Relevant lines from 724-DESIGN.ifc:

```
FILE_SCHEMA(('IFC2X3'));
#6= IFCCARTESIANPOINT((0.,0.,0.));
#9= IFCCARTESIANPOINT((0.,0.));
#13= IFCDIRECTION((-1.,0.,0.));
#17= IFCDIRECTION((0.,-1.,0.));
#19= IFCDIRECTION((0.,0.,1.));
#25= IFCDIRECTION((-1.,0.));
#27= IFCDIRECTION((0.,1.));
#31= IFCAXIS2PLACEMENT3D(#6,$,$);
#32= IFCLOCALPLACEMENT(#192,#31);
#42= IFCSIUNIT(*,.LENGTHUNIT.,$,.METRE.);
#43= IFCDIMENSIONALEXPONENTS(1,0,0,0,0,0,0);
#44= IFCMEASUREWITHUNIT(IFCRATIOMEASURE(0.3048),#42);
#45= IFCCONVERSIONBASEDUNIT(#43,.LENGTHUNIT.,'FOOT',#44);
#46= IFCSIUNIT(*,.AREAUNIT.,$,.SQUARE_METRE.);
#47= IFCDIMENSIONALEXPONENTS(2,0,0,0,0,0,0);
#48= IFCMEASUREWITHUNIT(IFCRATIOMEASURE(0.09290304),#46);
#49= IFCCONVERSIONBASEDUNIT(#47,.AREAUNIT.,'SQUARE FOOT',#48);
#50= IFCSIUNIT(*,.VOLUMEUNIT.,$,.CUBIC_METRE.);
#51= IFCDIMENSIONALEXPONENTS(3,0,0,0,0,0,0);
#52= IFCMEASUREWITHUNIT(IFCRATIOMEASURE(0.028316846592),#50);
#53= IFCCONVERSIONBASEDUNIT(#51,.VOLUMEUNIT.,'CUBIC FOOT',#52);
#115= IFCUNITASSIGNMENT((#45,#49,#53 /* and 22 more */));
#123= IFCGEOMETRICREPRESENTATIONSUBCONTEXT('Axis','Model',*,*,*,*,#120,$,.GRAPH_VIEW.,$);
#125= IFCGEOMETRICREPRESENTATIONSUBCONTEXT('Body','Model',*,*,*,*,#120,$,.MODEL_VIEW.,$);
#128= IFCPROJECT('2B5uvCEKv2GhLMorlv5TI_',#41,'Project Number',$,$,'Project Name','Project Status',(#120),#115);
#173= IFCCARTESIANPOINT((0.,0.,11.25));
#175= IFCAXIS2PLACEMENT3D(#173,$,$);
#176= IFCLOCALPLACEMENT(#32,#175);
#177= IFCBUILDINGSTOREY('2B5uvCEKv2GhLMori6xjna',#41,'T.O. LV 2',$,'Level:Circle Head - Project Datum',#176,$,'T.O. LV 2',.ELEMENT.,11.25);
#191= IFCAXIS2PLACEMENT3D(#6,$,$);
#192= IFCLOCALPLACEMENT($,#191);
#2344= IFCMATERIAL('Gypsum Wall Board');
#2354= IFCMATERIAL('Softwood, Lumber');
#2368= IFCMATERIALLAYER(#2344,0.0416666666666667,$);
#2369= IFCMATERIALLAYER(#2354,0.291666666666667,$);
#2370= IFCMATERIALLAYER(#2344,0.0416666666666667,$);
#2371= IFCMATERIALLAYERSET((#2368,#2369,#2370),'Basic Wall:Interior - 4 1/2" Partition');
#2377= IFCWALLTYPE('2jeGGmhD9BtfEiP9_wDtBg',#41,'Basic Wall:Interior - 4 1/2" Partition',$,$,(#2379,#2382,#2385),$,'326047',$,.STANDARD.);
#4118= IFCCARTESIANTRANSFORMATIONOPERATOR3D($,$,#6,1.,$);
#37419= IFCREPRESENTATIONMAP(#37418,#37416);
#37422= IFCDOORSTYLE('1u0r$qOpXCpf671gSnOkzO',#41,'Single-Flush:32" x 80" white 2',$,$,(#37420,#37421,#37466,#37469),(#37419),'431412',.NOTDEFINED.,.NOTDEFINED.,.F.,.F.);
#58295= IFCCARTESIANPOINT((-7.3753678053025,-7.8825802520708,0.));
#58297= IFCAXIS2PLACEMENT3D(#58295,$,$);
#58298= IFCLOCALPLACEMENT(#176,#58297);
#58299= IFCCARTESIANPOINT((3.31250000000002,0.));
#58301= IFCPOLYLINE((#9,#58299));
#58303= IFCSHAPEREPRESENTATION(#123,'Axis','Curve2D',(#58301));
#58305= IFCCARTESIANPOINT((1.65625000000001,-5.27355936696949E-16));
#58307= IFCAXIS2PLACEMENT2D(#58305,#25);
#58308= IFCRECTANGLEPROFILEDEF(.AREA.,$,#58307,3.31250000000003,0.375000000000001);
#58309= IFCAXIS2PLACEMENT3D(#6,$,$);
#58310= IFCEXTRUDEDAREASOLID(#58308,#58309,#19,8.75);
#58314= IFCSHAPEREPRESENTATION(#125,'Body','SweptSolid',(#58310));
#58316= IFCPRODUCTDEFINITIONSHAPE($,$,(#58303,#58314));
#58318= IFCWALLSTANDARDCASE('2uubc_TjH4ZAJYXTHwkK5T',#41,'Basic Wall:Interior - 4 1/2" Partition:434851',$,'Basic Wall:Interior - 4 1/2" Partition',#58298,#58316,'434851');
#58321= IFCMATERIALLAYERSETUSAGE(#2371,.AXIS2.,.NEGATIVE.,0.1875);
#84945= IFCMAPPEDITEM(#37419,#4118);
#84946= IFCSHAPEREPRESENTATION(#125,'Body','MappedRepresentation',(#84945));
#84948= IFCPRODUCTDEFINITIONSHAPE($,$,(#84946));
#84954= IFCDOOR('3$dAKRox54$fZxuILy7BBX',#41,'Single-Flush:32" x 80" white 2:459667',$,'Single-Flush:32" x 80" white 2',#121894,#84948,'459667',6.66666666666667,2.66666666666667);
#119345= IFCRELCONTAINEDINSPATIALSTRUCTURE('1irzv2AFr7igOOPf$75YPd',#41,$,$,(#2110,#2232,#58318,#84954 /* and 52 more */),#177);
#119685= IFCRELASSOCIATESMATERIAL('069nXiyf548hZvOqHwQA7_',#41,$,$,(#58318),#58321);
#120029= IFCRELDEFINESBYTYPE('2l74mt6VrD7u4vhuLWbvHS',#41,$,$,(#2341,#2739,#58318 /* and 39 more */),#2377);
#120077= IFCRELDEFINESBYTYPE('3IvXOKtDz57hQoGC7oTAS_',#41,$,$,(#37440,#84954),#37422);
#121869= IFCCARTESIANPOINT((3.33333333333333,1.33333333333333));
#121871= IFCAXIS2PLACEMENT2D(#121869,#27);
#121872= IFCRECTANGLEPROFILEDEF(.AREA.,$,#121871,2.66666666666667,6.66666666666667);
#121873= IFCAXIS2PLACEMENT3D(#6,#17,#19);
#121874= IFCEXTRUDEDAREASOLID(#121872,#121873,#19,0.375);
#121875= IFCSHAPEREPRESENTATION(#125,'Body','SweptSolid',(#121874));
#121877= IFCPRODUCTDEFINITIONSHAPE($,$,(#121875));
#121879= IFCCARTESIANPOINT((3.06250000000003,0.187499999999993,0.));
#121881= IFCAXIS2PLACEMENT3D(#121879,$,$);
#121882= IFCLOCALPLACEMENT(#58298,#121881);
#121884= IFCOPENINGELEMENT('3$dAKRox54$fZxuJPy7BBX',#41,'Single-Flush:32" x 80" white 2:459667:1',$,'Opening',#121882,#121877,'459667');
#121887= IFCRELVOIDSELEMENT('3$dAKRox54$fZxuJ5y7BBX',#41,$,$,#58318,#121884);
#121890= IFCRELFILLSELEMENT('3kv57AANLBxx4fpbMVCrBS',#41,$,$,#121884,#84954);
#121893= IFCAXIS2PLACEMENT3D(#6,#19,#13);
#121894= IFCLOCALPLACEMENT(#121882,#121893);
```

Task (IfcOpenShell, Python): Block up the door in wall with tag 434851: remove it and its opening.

```python
import ifcopenshell
import ifcopenshell.api.feature
import ifcopenshell.api.root
import ifcopenshell.geom
import ifcopenshell.util.shape

model = ifcopenshell.open("724-DESIGN.ifc")
settings = ifcopenshell.geom.settings()


def volume(element):
    """Net volume in cubic metres, openings subtracted."""
    shape = ifcopenshell.geom.create_shape(settings, element)
    return ifcopenshell.util.shape.get_volume(shape.geometry)


door = model.by_guid("3$dAKRox54$fZxuILy7BBX")
opening = door.FillsVoids[0].RelatingOpeningElement
wall = opening.VoidsElements[0].RelatingBuildingElement
before = volume(wall)

ifcopenshell.api.root.remove_product(model, product=door)
ifcopenshell.api.feature.remove_feature(model, feature=opening)

after = volume(wall)

print(f"wall volume {before:.3f} -> {after:.3f} m3")

model.write("724-DESIGN-out.ifc")
```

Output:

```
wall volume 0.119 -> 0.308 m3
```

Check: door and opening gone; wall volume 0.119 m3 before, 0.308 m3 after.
